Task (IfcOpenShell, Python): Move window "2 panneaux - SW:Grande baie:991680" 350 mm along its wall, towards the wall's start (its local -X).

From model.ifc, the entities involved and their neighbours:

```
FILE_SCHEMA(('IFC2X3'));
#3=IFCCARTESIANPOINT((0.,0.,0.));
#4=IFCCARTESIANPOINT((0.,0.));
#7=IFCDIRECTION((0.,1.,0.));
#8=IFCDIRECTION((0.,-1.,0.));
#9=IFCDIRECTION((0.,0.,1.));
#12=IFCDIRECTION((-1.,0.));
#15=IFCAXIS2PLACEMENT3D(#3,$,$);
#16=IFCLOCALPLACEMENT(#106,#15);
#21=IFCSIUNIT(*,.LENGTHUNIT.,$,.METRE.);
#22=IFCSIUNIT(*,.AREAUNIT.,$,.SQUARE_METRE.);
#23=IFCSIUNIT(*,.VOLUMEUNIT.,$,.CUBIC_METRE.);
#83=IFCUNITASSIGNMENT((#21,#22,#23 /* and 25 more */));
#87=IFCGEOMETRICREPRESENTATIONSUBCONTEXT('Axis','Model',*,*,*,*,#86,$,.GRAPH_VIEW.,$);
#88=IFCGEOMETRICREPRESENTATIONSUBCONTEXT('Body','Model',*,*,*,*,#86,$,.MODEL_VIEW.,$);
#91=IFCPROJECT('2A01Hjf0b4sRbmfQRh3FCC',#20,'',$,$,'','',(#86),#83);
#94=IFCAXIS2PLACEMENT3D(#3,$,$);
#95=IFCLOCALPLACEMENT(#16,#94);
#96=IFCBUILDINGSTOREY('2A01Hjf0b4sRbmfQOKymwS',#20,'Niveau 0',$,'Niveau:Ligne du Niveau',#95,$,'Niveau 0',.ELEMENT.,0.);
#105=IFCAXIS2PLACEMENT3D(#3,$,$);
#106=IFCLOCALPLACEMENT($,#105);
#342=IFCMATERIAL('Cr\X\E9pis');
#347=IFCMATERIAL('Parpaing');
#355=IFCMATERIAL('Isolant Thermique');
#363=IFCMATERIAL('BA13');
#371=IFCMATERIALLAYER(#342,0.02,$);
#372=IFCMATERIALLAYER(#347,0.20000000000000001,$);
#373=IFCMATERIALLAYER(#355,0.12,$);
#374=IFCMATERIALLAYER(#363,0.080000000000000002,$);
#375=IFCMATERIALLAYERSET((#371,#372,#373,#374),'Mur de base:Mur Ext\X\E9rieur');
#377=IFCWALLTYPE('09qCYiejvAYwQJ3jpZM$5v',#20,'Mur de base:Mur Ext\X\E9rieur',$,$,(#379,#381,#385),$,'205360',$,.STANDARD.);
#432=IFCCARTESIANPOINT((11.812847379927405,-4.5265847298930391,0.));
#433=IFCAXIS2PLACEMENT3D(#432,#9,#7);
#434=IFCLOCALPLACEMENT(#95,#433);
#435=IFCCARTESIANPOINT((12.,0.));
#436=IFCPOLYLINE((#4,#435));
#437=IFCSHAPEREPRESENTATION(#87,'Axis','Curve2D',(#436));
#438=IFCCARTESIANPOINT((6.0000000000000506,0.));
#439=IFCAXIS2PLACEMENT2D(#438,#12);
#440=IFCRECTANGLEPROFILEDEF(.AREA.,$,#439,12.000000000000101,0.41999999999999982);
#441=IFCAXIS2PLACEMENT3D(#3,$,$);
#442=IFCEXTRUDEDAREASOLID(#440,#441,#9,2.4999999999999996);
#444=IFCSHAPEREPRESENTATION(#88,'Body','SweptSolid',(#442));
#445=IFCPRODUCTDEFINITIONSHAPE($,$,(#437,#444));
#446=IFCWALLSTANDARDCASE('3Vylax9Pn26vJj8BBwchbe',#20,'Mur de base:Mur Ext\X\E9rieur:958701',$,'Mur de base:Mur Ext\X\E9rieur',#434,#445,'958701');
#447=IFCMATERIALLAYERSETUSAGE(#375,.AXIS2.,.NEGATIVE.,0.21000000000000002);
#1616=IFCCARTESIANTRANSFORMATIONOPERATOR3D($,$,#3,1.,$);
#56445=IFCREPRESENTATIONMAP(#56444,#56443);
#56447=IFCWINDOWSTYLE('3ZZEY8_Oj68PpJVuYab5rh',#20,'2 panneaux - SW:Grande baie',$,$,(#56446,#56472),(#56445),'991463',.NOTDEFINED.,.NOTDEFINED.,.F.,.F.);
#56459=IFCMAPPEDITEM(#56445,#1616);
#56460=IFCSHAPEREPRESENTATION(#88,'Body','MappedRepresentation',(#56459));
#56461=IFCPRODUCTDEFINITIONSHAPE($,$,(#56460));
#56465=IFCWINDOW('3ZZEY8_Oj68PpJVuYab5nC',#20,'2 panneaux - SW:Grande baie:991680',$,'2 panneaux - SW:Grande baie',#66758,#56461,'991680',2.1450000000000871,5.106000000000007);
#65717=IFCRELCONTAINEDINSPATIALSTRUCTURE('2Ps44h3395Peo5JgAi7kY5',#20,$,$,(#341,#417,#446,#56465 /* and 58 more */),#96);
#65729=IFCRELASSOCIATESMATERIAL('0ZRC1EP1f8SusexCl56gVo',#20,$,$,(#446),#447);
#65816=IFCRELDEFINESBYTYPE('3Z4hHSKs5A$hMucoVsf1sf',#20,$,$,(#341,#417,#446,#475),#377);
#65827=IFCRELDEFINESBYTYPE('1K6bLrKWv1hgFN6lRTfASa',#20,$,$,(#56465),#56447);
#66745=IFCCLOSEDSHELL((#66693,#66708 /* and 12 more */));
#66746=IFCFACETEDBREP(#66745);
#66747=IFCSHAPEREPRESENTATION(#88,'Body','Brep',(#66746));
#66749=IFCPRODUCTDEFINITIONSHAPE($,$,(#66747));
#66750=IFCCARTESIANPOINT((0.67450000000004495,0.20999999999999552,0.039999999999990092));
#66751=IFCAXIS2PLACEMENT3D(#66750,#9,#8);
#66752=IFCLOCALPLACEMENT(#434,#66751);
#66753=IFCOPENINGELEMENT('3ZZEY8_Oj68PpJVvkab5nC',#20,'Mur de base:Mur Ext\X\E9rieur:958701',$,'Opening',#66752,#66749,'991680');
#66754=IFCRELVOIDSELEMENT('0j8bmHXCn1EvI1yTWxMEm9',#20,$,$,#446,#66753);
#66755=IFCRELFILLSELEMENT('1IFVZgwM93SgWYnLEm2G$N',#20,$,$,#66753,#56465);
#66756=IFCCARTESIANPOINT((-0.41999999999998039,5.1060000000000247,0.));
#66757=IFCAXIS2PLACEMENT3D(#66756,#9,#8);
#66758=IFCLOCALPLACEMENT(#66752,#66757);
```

```python
import ifcopenshell
import ifcopenshell.api.geometry
import ifcopenshell.util.placement
import ifcopenshell.util.unit

model = ifcopenshell.open("model.ifc")
unit_scale = ifcopenshell.util.unit.calculate_unit_scale(model)

window = model.by_guid("3ZZEY8_Oj68PpJVuYab5nC")
opening = window.FillsVoids[0].RelatingOpeningElement
wall = opening.VoidsElements[0].RelatingBuildingElement

wall_matrix = ifcopenshell.util.placement.get_local_placement(wall.ObjectPlacement)
shift = wall_matrix[:3, 0] * -0.35 / unit_scale
before = ifcopenshell.util.placement.get_local_placement(window.ObjectPlacement)[:3, 3].copy()

# The window is placed relative to its opening, so it follows when the opening moves.
matrix = ifcopenshell.util.placement.get_local_placement(opening.ObjectPlacement)
matrix[:3, 3] += shift
ifcopenshell.api.geometry.edit_object_placement(
    model, product=opening, matrix=matrix, is_si=False, should_transform_children=True
)

after = ifcopenshell.util.placement.get_local_placement(window.ObjectPlacement)[:3, 3]
print("window moved by", (after - before).round(3) + 0.0)

model.write("model-out.ifc")
```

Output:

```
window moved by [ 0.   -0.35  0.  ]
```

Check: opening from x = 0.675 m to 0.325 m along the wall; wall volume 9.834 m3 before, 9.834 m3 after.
